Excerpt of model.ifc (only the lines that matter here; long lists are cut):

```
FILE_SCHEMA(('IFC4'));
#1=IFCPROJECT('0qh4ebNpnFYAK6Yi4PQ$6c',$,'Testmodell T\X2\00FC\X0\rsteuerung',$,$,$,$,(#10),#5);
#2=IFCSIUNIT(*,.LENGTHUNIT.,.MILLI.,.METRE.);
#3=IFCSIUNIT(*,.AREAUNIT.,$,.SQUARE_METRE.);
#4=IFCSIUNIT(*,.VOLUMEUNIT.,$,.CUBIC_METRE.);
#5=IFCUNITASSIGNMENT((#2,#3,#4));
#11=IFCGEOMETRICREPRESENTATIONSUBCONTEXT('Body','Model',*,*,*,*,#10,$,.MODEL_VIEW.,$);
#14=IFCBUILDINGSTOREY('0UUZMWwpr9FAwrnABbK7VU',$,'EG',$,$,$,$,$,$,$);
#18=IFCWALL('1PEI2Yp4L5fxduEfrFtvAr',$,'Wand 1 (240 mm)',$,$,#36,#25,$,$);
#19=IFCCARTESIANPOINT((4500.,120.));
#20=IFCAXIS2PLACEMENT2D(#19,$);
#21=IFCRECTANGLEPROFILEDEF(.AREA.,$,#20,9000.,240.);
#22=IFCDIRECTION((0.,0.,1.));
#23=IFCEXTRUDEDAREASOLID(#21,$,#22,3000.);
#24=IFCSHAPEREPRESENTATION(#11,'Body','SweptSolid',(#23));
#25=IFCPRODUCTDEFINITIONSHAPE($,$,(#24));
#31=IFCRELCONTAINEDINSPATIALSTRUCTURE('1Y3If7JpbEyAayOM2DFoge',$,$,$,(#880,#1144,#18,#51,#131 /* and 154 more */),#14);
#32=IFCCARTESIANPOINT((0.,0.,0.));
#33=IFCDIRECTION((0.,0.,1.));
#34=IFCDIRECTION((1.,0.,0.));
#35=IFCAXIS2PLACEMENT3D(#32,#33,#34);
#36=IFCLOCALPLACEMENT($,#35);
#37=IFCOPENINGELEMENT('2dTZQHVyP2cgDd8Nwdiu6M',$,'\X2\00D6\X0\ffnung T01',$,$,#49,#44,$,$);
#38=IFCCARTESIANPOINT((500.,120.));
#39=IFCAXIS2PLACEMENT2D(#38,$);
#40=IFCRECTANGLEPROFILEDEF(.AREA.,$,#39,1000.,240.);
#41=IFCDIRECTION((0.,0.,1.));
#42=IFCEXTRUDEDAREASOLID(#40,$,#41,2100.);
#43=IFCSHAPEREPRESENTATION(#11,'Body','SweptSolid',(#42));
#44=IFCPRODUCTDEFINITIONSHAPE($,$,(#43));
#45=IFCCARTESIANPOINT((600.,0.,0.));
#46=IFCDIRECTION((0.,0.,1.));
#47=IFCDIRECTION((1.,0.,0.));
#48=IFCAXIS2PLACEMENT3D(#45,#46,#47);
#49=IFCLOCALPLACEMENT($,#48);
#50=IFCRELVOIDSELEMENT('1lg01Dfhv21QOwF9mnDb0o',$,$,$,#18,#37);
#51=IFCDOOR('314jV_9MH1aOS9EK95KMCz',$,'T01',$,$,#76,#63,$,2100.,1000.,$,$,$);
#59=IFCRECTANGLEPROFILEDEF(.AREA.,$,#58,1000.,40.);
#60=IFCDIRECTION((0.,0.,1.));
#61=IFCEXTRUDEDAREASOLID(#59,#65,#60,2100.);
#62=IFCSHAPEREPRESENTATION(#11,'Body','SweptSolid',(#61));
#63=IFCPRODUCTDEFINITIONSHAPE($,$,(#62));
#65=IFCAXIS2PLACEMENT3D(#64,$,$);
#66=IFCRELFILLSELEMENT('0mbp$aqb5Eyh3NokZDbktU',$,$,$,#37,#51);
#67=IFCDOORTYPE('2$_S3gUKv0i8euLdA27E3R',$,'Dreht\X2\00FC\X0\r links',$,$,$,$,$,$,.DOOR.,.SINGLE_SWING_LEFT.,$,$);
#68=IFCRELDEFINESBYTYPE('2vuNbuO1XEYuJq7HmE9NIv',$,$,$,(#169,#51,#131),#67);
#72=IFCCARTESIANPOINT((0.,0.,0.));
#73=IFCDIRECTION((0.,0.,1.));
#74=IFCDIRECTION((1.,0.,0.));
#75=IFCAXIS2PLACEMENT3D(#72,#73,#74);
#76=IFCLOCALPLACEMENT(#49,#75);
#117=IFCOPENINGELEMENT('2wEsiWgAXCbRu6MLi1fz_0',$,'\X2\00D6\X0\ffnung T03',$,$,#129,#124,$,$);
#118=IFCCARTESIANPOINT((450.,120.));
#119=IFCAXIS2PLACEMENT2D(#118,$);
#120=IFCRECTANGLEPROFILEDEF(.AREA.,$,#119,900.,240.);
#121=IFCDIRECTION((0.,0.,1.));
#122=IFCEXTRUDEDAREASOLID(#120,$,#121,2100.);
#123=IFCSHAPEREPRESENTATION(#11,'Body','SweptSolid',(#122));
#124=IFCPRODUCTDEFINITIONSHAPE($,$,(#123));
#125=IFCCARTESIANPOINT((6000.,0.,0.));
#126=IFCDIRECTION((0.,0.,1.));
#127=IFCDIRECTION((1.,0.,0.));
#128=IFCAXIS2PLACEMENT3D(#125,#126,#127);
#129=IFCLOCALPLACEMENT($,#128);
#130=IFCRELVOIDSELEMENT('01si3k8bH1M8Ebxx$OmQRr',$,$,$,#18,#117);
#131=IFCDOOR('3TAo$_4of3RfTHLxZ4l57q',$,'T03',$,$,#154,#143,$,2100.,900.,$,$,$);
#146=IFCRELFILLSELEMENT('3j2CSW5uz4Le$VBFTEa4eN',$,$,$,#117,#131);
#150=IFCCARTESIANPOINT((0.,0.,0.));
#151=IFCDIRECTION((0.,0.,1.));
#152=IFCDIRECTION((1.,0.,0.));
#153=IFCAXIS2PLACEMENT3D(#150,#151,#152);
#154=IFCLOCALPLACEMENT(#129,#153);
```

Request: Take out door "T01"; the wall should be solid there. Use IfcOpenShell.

```python
import ifcopenshell
import ifcopenshell.api.feature
import ifcopenshell.api.root
import ifcopenshell.geom
import ifcopenshell.util.shape

model = ifcopenshell.open("model.ifc")
settings = ifcopenshell.geom.settings()


def volume(element):
    """Net volume in cubic metres, openings subtracted."""
    shape = ifcopenshell.geom.create_shape(settings, element)
    return ifcopenshell.util.shape.get_volume(shape.geometry)


door = model.by_guid("314jV_9MH1aOS9EK95KMCz")
opening = door.FillsVoids[0].RelatingOpeningElement
wall = opening.VoidsElements[0].RelatingBuildingElement
before = volume(wall)

ifcopenshell.api.root.remove_product(model, product=door)
ifcopenshell.api.feature.remove_feature(model, feature=opening)

after = volume(wall)

print(f"wall volume {before:.3f} -> {after:.3f} m3")

model.write("model_edited.ifc")
```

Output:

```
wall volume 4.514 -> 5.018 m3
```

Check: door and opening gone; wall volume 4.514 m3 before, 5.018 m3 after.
